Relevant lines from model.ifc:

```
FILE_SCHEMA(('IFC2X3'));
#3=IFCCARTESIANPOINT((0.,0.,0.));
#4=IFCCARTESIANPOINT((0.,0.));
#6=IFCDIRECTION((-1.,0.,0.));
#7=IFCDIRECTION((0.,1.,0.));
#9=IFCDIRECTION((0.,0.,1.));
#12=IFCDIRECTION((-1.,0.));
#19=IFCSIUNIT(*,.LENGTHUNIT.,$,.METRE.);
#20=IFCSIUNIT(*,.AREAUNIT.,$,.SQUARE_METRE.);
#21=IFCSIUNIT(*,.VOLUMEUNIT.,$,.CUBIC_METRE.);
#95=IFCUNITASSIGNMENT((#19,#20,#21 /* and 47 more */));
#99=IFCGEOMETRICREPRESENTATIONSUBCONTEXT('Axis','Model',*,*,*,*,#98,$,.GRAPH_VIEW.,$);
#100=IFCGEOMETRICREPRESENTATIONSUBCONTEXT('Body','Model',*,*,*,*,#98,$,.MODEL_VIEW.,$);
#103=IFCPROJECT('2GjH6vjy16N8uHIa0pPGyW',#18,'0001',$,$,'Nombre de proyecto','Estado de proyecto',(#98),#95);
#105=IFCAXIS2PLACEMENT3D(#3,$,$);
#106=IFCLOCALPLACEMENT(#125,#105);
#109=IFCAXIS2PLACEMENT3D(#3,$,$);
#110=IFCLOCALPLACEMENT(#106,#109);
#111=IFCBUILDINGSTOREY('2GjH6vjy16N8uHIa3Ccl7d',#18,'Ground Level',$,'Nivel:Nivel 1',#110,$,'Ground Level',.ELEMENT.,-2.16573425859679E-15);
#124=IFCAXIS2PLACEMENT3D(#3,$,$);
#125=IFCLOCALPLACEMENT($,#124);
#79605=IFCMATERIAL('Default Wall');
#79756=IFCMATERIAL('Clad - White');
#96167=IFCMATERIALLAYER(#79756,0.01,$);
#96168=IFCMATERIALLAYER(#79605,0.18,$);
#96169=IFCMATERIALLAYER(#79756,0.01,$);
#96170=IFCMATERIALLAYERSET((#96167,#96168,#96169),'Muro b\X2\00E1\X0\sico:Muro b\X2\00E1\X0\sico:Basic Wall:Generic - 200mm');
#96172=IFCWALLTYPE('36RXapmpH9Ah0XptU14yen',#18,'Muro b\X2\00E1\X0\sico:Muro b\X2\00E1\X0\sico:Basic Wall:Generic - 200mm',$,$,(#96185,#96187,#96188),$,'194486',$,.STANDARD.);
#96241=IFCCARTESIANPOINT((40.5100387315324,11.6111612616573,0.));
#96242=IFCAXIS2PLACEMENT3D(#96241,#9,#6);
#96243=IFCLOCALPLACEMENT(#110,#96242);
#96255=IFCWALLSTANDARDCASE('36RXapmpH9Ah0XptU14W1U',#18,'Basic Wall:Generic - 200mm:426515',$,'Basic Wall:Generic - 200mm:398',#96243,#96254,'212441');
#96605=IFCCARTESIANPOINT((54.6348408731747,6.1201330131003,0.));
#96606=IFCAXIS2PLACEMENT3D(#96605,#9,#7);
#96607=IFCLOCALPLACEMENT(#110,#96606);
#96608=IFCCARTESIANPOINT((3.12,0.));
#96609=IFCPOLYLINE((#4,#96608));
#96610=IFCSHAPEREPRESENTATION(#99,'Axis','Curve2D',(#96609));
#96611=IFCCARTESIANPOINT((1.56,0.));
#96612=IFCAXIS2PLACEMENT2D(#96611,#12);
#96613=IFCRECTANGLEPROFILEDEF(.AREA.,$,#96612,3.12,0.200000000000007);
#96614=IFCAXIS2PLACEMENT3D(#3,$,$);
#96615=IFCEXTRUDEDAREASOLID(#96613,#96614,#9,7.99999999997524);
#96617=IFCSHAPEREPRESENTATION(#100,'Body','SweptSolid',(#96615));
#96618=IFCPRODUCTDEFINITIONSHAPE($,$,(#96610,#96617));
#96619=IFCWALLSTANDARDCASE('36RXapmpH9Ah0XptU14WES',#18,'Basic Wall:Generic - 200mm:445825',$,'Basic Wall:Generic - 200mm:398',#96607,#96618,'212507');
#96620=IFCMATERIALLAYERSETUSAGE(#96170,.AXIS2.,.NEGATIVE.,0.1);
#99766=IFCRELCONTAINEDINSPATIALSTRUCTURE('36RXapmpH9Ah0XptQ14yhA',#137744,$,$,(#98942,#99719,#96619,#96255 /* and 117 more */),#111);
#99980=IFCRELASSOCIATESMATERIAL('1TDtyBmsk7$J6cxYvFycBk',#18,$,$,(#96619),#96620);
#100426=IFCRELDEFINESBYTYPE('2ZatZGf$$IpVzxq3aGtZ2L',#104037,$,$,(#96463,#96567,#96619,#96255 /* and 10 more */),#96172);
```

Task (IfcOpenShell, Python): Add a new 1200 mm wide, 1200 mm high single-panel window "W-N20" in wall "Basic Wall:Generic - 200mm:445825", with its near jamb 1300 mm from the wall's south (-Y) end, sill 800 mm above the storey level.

```python
import numpy as np
import ifcopenshell
import ifcopenshell.api.feature
import ifcopenshell.api.geometry
import ifcopenshell.api.root
import ifcopenshell.api.spatial
import ifcopenshell.api.type
import ifcopenshell.geom
import ifcopenshell.util.element
import ifcopenshell.util.placement
import ifcopenshell.util.representation
import ifcopenshell.util.shape
import ifcopenshell.util.unit

model = ifcopenshell.open("model.ifc")
unit_scale = ifcopenshell.util.unit.calculate_unit_scale(model)
settings = ifcopenshell.geom.settings()


def volume(element):
    """Net volume in cubic metres, openings subtracted."""
    shape = ifcopenshell.geom.create_shape(settings, element)
    return ifcopenshell.util.shape.get_volume(shape.geometry)


wall = model.by_guid("36RXapmpH9Ah0XptU14WES")
storey = ifcopenshell.util.element.get_container(wall, ifc_class="IfcBuildingStorey")
context = ifcopenshell.util.representation.get_context(model, "Model", "Body", "MODEL_VIEW")
before = volume(wall)

width, height, from_end, sill = 1.2, 1.2, 1.3, 0.8  # metres

# The wall runs along its own X axis, and the end named is its -X end.
wall_shape = ifcopenshell.geom.create_shape(settings, wall)
x, y, z = ifcopenshell.util.shape.get_vertices(wall_shape.geometry).T
start = x.min() + from_end
face, thickness = float(y.min()), float(y.max() - y.min())
wall_matrix = ifcopenshell.util.placement.get_local_placement(wall.ObjectPlacement)
level = ifcopenshell.util.placement.get_local_placement(storey.ObjectPlacement)[2, 3]


def in_wall(x, y):
    """Placement at x, y metres in the wall's axes, at sill height."""
    matrix = wall_matrix.copy()
    matrix[:, 3] = wall_matrix @ np.array([x / unit_scale, y / unit_scale, 0.0, 1.0])
    matrix[2, 3] = level + sill / unit_scale
    return matrix


# Opening: a box that overshoots both wall faces by 50 mm.
opening = ifcopenshell.api.root.create_entity(model, ifc_class="IfcOpeningElement")
box = ifcopenshell.api.geometry.add_wall_representation(
    model, context=context, length=width, height=height, thickness=thickness + 0.1
)
ifcopenshell.api.geometry.assign_representation(model, product=opening, representation=box)
ifcopenshell.api.geometry.edit_object_placement(model, product=opening, matrix=in_wall(start, face - 0.05), is_si=False)
ifcopenshell.api.feature.add_feature(model, feature=opening, element=wall)

window = ifcopenshell.api.root.create_entity(model, ifc_class="IfcWindow", name="W-N20")
window.OverallWidth, window.OverallHeight = width / unit_scale, height / unit_scale
body = ifcopenshell.api.geometry.add_window_representation(
    model,
    context=context,
    overall_width=window.OverallWidth,
    overall_height=window.OverallHeight,
    partition_type="SINGLE_PANEL",
)
ifcopenshell.api.geometry.assign_representation(model, product=window, representation=body)
ifcopenshell.api.spatial.assign_container(model, products=[window], relating_structure=storey)
fills = ifcopenshell.api.feature.add_filling(model, opening=opening, element=window)
fills.OwnerHistory = window.OwnerHistory  # required in IFC2X3

# IFC2X3 keeps the operation on the window style.
style = ifcopenshell.api.root.create_entity(model, ifc_class="IfcWindowStyle", name="W-N20")
style.OperationType, style.ConstructionType = "SINGLE_PANEL", "NOTDEFINED"
style.ParameterTakesPrecedence = style.Sizeable = False
ifcopenshell.api.type.assign_type(model, related_objects=[window], relating_type=style)

# Centre the window in the wall's thickness.
ifcopenshell.api.geometry.edit_object_placement(model, product=window, matrix=in_wall(start, face), is_si=False)
window_shape = ifcopenshell.geom.create_shape(settings, window)
depth = ifcopenshell.util.shape.get_vertices(window_shape.geometry)[:, 1]
offset = face + thickness / 2 - (depth.min() + depth.max()) / 2
ifcopenshell.api.geometry.edit_object_placement(model, product=window, matrix=in_wall(start, offset), is_si=False)

after = volume(wall)

print(f"wall volume {before:.3f} -> {after:.3f} m3")

model.write("model_v2.ifc")
```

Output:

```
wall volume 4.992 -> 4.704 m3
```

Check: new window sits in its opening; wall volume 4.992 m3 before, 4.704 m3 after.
